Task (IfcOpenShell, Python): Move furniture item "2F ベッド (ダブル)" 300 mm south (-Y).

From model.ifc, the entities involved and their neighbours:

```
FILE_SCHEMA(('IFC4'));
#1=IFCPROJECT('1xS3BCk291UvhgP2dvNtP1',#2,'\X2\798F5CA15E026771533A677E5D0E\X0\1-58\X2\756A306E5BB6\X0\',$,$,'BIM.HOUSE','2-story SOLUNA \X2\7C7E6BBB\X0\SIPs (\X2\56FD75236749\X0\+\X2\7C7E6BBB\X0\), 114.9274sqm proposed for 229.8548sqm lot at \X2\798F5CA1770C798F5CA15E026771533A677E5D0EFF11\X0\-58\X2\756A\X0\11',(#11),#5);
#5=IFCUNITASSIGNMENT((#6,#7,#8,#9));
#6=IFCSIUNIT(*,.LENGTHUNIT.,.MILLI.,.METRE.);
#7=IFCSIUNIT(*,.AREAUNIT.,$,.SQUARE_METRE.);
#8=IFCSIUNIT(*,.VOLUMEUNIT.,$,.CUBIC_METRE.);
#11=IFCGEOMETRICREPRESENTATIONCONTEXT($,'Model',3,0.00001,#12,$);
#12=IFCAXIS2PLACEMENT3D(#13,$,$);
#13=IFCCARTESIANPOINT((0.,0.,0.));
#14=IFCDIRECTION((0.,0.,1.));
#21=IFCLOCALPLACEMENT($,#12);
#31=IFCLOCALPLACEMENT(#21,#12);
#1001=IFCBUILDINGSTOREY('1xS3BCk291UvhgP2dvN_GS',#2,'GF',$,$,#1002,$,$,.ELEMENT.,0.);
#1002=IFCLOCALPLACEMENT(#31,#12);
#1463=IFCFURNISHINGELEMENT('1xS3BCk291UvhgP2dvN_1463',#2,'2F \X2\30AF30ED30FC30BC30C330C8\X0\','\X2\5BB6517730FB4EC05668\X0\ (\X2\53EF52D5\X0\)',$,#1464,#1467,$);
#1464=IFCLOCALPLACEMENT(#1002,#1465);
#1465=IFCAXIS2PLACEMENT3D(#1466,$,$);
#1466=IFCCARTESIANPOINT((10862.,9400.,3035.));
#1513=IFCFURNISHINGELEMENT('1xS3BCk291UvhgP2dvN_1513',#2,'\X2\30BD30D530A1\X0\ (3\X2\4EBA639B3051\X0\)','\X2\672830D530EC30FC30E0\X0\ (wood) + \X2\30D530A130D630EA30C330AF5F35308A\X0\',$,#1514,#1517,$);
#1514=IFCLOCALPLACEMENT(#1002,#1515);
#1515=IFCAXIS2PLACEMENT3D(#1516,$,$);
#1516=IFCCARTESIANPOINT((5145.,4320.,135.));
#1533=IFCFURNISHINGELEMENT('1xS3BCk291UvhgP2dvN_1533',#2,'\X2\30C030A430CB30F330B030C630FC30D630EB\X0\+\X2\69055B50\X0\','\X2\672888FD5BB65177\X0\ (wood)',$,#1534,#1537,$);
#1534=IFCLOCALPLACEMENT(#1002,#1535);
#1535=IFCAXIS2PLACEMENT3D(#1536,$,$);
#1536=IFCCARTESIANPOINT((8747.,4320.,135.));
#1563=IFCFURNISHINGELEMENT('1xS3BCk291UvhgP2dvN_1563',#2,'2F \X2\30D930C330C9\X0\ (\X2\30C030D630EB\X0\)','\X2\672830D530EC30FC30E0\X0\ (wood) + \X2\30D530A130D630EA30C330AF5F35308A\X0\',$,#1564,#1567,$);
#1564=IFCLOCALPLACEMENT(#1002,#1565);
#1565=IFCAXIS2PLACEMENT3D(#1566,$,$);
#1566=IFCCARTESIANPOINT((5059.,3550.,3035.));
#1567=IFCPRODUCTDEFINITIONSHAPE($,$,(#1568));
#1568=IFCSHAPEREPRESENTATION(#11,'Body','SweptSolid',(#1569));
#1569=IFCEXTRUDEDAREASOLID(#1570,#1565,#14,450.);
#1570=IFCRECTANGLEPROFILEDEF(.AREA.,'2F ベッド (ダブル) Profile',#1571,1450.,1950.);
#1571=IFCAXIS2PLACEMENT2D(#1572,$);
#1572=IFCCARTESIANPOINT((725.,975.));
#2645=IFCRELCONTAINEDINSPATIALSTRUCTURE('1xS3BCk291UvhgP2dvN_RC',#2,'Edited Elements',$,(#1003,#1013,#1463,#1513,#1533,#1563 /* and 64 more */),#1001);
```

```python
import ifcopenshell
import ifcopenshell.api.geometry
import ifcopenshell.util.placement

model = ifcopenshell.open("model.ifc")

item = model.by_guid("1xS3BCk291UvhgP2dvN_1563")
matrix = ifcopenshell.util.placement.get_local_placement(item.ObjectPlacement)
matrix[1, 3] -= 300.0
ifcopenshell.api.geometry.edit_object_placement(model, product=item, matrix=matrix, is_si=False)

print(ifcopenshell.util.placement.get_local_placement(item.ObjectPlacement).round(3) + 0.0)

model.write("model_edited.ifc")
```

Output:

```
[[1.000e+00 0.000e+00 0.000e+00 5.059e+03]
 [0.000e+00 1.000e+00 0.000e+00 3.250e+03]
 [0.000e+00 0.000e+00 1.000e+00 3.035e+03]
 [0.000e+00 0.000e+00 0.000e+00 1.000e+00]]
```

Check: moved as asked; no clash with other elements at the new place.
